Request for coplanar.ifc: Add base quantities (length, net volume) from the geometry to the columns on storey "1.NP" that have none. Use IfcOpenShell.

First a look at what the model holds.

```python
import ifcopenshell
import ifcopenshell.util.element
import ifcopenshell.util.unit

model = ifcopenshell.open("coplanar.ifc")
print(model.schema)
for unit_type in ("LENGTHUNIT", "AREAUNIT", "VOLUMEUNIT"):
    print(unit_type, ifcopenshell.util.unit.calculate_unit_scale(model, unit_type))
storey = next(s for s in model.by_type("IfcBuildingStorey") if s.Name == "1.NP")
columns = [e for e in ifcopenshell.util.element.get_decomposition(storey) if e.is_a("IfcColumn")]
for e in sorted(columns, key=lambda e: e.id()):
    print(e.id(), e.is_a(), e.Name, list(ifcopenshell.util.element.get_psets(e, qtos_only=True)), sep=" | ")
```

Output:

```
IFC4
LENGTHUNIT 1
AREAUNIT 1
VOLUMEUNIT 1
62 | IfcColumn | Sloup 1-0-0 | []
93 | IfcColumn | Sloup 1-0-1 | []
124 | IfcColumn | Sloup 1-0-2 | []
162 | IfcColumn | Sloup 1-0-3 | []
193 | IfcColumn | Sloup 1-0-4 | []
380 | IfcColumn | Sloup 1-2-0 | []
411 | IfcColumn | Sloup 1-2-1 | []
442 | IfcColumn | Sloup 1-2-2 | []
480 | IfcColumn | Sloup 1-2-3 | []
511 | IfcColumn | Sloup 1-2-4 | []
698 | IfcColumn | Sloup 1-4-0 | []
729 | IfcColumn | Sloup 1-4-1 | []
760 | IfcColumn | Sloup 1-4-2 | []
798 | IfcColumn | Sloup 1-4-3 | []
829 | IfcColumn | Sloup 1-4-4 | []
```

```python
import ifcopenshell
import ifcopenshell.api.pset
import ifcopenshell.geom
import ifcopenshell.util.element
import ifcopenshell.util.shape
import ifcopenshell.util.unit

model = ifcopenshell.open("coplanar.ifc")
unit_scale = ifcopenshell.util.unit.calculate_unit_scale(model)
volume_scale = ifcopenshell.util.unit.calculate_unit_scale(model, "VOLUMEUNIT")
settings = ifcopenshell.geom.settings()

storey = next(s for s in model.by_type("IfcBuildingStorey") if s.Name == "1.NP")
columns = [e for e in ifcopenshell.util.element.get_decomposition(storey) if e.is_a("IfcColumn")]

for e in sorted(columns, key=lambda e: e.id()):
    if ifcopenshell.util.element.get_psets(e, qtos_only=True, should_inherit=False):
        continue
    # Geometry comes back in metres, in the element's own axes.
    shape = ifcopenshell.geom.create_shape(settings, e)
    values = {
        "Length": ifcopenshell.util.shape.get_z(shape.geometry) / unit_scale,
        "NetVolume": ifcopenshell.util.shape.get_volume(shape.geometry) / volume_scale,
    }
    qto = ifcopenshell.api.pset.add_qto(model, product=e, name="Qto_ColumnBaseQuantities")
    ifcopenshell.api.pset.edit_qto(model, qto=qto, properties=values)
    print(e.id(), {k: round(v, 3) for k, v in values.items()})

model.write("coplanar_edited.ifc")
```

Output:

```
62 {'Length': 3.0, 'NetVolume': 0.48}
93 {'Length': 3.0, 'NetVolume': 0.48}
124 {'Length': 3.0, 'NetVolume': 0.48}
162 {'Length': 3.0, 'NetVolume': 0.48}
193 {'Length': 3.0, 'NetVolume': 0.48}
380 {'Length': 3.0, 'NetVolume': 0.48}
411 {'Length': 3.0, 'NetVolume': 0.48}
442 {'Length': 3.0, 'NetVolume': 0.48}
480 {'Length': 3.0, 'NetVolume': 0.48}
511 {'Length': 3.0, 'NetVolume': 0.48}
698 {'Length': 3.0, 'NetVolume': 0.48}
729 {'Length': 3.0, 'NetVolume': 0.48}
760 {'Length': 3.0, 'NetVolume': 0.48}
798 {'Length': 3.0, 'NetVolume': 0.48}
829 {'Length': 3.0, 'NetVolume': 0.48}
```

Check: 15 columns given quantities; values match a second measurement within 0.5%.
